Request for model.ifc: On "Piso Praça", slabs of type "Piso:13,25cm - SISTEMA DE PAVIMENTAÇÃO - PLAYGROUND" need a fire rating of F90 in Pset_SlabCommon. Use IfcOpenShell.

First a look at what the model holds.

```python
import ifcopenshell
import ifcopenshell.util.element

model = ifcopenshell.open("model.ifc")
print(model.schema)
storey = next(s for s in model.by_type("IfcBuildingStorey") if s.Name == "Piso Praça")
slabs = [e for e in ifcopenshell.util.element.get_decomposition(storey) if e.is_a("IfcSlab")]
seen = {}
for e in slabs:
    element_type = ifcopenshell.util.element.get_type(e)
    key = (element_type.Name if element_type != e and element_type else None, ifcopenshell.util.element.get_pset(e, "Pset_SlabCommon", "FireRating"))
    seen[key] = seen.get(key, 0) + 1
for (name, value), count in sorted(seen.items(), key=str):
    print(count, "x", name, "|", value)
```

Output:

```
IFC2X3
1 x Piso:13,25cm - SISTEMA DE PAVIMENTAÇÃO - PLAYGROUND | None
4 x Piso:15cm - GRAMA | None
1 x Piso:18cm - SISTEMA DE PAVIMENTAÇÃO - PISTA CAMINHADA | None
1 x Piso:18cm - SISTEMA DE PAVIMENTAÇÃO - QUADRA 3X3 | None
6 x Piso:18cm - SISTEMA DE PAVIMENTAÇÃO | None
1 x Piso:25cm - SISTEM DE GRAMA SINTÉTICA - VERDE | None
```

```python
import ifcopenshell
import ifcopenshell.api.pset
import ifcopenshell.util.element

model = ifcopenshell.open("model.ifc")

storey = next(s for s in model.by_type("IfcBuildingStorey") if s.Name == "Piso Praça")
slabs = [e for e in ifcopenshell.util.element.get_decomposition(storey) if e.is_a("IfcSlab")]

count = 0
for e in slabs:
    element_type = ifcopenshell.util.element.get_type(e)
    if element_type in (None, e) or element_type.Name != "Piso:13,25cm - SISTEMA DE PAVIMENTAÇÃO - PLAYGROUND":
        continue
    # add_pset returns the element's existing set when there is one.
    pset = ifcopenshell.api.pset.add_pset(model, product=e, name="Pset_SlabCommon")
    ifcopenshell.api.pset.edit_pset(model, pset=pset, properties={"FireRating": "F90"})
    count += 1

print(count, "slabs updated")

model.write("model_v2.ifc")
```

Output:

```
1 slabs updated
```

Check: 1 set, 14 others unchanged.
